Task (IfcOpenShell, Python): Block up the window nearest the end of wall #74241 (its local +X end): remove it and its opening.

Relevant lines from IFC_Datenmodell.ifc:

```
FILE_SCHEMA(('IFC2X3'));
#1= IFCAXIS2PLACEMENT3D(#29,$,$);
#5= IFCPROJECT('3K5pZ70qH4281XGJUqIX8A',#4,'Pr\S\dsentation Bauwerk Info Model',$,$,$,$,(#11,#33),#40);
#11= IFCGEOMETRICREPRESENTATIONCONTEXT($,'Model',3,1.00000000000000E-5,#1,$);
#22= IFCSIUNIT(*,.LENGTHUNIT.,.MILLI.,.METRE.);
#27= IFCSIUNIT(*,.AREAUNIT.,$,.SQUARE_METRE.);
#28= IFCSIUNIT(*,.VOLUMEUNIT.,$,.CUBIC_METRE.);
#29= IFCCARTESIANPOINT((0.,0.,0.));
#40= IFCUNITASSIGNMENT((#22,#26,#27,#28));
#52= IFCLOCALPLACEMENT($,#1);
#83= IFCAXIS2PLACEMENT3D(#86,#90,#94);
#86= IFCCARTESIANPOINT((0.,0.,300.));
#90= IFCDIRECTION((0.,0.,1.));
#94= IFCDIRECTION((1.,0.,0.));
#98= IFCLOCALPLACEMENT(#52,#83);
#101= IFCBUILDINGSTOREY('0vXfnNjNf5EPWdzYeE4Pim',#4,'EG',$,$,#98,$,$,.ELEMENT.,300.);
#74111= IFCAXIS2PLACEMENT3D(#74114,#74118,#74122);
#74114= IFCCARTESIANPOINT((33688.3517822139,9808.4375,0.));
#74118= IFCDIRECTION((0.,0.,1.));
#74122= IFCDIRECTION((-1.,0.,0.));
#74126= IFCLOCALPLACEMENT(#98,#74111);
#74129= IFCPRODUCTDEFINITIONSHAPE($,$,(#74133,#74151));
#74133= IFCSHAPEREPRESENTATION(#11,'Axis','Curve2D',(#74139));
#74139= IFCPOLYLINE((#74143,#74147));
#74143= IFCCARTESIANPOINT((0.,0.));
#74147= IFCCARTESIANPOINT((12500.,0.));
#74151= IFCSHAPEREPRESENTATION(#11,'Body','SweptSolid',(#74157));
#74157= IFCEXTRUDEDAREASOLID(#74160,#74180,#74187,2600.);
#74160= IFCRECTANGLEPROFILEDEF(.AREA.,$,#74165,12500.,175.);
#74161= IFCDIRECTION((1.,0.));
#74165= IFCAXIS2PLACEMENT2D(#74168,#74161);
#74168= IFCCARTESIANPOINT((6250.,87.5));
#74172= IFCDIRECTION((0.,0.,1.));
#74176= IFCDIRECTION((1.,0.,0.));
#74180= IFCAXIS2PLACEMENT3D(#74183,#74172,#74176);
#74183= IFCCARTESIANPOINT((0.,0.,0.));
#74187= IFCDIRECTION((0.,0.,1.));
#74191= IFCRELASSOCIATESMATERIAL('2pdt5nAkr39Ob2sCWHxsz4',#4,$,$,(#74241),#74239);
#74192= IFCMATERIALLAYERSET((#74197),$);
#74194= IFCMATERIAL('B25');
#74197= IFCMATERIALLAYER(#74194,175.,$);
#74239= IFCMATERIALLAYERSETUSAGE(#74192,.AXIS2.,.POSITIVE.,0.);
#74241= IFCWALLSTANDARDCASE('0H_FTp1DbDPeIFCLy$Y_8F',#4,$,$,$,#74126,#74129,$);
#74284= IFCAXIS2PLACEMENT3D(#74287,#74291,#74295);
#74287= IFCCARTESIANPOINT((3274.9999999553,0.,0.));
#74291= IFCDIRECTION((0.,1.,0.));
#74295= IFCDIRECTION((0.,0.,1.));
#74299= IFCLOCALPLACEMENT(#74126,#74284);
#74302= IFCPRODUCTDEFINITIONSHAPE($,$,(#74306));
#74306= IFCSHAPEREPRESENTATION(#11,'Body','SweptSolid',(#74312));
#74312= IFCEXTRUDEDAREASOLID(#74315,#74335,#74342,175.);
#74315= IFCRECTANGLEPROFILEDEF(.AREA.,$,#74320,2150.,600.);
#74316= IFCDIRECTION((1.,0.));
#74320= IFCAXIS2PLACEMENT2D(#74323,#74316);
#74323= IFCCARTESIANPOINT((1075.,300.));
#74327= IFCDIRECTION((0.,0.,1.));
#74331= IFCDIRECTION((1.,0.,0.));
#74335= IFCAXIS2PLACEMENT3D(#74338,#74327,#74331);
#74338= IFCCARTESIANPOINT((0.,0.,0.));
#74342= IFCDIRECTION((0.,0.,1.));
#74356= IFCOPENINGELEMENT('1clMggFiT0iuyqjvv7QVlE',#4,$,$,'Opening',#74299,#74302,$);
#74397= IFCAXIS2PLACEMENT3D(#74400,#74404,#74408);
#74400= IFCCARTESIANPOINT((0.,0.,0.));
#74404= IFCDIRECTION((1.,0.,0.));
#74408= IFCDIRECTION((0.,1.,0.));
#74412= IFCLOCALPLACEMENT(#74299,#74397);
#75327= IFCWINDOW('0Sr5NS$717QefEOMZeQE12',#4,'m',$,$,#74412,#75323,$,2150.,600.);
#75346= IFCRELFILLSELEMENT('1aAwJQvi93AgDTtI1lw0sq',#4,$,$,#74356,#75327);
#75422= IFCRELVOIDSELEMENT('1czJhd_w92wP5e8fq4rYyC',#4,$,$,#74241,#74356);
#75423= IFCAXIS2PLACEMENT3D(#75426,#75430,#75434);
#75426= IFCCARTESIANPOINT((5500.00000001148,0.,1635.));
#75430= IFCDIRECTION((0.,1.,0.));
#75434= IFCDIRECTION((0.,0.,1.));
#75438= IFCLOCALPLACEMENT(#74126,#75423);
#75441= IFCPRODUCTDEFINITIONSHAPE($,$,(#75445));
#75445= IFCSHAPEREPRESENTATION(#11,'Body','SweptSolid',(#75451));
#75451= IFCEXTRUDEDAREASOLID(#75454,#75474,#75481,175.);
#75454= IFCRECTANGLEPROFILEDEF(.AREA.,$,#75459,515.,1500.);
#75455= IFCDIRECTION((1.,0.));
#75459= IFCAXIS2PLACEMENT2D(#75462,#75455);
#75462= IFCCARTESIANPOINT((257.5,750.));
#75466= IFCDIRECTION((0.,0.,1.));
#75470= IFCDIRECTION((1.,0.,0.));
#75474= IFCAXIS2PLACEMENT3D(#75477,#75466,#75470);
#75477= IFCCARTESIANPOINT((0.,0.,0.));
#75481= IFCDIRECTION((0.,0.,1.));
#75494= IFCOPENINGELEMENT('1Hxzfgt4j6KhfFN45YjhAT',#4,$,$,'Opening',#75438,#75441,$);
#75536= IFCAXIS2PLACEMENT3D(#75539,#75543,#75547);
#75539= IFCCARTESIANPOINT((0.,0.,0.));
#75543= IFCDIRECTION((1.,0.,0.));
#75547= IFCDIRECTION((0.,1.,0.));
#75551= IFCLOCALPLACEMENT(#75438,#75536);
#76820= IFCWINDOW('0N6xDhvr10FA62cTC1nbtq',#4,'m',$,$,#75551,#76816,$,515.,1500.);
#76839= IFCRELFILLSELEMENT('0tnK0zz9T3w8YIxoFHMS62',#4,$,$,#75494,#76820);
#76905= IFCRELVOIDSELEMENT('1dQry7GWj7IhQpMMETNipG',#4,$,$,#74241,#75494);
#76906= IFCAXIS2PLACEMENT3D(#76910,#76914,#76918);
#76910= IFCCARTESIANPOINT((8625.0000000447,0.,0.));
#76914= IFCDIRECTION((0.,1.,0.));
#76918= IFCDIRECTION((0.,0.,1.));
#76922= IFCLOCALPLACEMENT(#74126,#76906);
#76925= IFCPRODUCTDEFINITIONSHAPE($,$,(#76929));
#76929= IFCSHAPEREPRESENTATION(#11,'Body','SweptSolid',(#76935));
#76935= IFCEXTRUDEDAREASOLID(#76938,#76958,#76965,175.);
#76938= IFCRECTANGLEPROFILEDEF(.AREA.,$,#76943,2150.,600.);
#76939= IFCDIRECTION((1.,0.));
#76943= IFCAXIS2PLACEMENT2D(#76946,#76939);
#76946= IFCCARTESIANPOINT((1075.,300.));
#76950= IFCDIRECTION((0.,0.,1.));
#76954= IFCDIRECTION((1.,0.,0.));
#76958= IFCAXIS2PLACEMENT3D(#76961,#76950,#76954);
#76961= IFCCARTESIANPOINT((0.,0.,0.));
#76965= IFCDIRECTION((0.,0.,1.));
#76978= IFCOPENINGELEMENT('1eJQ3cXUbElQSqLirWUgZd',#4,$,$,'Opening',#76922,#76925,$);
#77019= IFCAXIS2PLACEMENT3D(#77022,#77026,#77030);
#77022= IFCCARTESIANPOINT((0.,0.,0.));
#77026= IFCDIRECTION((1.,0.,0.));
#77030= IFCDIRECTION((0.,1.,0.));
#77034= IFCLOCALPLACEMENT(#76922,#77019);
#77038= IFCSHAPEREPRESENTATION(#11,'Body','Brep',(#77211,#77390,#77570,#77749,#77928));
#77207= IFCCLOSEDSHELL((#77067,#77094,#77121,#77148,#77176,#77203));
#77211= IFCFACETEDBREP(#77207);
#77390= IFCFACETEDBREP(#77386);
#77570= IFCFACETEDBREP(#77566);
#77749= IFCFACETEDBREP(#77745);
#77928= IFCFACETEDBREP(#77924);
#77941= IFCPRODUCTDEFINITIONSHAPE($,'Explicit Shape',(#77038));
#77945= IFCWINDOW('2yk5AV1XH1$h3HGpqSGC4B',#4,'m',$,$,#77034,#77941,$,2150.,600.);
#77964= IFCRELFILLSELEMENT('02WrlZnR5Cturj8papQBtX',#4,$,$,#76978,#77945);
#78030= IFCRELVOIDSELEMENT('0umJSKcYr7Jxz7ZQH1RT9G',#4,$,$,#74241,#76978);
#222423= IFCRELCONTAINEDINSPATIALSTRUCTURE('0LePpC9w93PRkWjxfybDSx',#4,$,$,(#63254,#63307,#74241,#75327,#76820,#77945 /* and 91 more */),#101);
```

```python
import ifcopenshell
import ifcopenshell.api.feature
import ifcopenshell.api.root
import ifcopenshell.geom
import ifcopenshell.util.shape

model = ifcopenshell.open("IFC_Datenmodell.ifc")
settings = ifcopenshell.geom.settings()


def volume(element):
    """Net volume in cubic metres, openings subtracted."""
    shape = ifcopenshell.geom.create_shape(settings, element)
    return ifcopenshell.util.shape.get_volume(shape.geometry)


window = model.by_id(77945)
opening = window.FillsVoids[0].RelatingOpeningElement
wall = opening.VoidsElements[0].RelatingBuildingElement
before = volume(wall)

ifcopenshell.api.root.remove_product(model, product=window)
ifcopenshell.api.feature.remove_feature(model, feature=opening)

after = volume(wall)

print(f"wall volume {before:.3f} -> {after:.3f} m3")

model.write("IFC_Datenmodell_rev.ifc")
```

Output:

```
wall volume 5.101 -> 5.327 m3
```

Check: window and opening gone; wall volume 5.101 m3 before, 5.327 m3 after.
